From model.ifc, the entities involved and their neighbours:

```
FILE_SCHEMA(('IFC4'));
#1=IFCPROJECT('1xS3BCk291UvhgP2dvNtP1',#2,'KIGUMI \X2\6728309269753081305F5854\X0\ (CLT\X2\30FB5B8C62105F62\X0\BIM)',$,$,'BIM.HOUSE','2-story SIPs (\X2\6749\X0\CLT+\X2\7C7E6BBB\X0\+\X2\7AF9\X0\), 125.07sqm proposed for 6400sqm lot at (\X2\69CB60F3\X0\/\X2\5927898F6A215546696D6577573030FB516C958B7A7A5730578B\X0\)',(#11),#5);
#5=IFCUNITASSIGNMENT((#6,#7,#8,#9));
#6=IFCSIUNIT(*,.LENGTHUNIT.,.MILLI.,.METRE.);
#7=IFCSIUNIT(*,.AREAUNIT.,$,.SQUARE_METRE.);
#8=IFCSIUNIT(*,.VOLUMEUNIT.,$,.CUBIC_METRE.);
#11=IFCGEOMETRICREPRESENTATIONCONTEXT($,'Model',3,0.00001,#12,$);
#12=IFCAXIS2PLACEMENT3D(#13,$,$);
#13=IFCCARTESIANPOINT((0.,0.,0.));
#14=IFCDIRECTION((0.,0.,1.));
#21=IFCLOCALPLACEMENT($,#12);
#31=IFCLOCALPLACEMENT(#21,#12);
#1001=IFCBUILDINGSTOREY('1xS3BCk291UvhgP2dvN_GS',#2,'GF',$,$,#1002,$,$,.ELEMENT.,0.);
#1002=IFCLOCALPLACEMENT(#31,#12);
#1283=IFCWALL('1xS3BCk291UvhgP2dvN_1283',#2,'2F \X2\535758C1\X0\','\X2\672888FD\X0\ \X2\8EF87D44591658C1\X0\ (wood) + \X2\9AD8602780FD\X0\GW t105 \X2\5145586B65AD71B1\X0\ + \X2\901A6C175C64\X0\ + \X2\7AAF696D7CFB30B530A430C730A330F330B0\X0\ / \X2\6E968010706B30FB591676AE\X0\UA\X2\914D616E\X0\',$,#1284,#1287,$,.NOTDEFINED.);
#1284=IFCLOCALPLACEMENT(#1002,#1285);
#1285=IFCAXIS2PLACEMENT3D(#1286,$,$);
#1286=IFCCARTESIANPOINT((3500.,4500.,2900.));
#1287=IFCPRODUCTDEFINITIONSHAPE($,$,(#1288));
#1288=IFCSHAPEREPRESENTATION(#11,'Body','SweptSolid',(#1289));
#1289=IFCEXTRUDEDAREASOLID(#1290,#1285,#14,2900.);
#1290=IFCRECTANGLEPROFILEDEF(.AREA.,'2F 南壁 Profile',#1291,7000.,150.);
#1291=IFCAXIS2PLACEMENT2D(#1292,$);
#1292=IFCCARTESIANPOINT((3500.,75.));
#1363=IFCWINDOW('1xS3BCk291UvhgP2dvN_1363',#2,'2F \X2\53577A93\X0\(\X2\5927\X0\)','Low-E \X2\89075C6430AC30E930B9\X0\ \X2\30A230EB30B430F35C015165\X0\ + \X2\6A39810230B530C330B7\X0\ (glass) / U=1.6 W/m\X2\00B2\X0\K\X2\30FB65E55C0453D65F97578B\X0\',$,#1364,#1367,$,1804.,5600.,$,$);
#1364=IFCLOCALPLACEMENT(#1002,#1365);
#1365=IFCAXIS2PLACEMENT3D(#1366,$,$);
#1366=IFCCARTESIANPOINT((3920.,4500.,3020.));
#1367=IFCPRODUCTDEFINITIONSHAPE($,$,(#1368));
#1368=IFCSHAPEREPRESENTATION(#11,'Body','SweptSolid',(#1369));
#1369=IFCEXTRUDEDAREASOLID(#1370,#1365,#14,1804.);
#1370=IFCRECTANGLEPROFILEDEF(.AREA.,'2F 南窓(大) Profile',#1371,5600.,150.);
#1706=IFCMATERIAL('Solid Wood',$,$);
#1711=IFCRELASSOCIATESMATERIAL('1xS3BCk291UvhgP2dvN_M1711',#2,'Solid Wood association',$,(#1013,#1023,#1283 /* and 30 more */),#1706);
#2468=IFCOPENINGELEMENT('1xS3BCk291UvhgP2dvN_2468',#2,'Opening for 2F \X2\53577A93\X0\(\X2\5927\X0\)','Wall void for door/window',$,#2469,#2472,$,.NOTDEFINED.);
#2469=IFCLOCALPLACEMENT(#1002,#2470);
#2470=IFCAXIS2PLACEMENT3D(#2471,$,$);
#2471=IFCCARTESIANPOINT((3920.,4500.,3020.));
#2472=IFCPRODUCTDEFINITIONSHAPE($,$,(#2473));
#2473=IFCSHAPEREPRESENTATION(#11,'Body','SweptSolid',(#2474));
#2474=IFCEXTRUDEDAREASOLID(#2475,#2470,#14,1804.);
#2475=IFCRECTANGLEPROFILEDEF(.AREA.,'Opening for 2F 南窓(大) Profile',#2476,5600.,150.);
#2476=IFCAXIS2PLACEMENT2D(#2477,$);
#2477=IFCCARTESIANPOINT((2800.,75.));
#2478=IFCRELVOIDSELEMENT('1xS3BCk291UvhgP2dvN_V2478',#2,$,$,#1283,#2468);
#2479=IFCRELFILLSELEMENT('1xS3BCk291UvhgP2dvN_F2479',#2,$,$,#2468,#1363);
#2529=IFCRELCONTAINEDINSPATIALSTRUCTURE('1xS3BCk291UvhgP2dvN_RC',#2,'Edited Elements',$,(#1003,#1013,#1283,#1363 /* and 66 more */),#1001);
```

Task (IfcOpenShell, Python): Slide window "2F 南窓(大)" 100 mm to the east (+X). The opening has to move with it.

```python
import ifcopenshell
import ifcopenshell.api.geometry
import ifcopenshell.util.placement
import ifcopenshell.util.unit

model = ifcopenshell.open("model.ifc")
unit_scale = ifcopenshell.util.unit.calculate_unit_scale(model)

window = model.by_guid("1xS3BCk291UvhgP2dvN_1363")
opening = window.FillsVoids[0].RelatingOpeningElement
wall = opening.VoidsElements[0].RelatingBuildingElement

wall_matrix = ifcopenshell.util.placement.get_local_placement(wall.ObjectPlacement)
shift = wall_matrix[:3, 0] * 0.1 / unit_scale
before = ifcopenshell.util.placement.get_local_placement(window.ObjectPlacement)[:3, 3].copy()

# The window is not placed relative to its opening, so move both.
for product in (opening, window):
    matrix = ifcopenshell.util.placement.get_local_placement(product.ObjectPlacement)
    matrix[:3, 3] += shift
    ifcopenshell.api.geometry.edit_object_placement(model, product=product, matrix=matrix, is_si=False)

after = ifcopenshell.util.placement.get_local_placement(window.ObjectPlacement)[:3, 3]
print("window moved by", (after - before).round(3) + 0.0)

model.write("model_v2.ifc")
```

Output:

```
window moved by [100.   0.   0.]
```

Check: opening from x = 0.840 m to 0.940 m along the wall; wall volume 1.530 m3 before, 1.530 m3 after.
